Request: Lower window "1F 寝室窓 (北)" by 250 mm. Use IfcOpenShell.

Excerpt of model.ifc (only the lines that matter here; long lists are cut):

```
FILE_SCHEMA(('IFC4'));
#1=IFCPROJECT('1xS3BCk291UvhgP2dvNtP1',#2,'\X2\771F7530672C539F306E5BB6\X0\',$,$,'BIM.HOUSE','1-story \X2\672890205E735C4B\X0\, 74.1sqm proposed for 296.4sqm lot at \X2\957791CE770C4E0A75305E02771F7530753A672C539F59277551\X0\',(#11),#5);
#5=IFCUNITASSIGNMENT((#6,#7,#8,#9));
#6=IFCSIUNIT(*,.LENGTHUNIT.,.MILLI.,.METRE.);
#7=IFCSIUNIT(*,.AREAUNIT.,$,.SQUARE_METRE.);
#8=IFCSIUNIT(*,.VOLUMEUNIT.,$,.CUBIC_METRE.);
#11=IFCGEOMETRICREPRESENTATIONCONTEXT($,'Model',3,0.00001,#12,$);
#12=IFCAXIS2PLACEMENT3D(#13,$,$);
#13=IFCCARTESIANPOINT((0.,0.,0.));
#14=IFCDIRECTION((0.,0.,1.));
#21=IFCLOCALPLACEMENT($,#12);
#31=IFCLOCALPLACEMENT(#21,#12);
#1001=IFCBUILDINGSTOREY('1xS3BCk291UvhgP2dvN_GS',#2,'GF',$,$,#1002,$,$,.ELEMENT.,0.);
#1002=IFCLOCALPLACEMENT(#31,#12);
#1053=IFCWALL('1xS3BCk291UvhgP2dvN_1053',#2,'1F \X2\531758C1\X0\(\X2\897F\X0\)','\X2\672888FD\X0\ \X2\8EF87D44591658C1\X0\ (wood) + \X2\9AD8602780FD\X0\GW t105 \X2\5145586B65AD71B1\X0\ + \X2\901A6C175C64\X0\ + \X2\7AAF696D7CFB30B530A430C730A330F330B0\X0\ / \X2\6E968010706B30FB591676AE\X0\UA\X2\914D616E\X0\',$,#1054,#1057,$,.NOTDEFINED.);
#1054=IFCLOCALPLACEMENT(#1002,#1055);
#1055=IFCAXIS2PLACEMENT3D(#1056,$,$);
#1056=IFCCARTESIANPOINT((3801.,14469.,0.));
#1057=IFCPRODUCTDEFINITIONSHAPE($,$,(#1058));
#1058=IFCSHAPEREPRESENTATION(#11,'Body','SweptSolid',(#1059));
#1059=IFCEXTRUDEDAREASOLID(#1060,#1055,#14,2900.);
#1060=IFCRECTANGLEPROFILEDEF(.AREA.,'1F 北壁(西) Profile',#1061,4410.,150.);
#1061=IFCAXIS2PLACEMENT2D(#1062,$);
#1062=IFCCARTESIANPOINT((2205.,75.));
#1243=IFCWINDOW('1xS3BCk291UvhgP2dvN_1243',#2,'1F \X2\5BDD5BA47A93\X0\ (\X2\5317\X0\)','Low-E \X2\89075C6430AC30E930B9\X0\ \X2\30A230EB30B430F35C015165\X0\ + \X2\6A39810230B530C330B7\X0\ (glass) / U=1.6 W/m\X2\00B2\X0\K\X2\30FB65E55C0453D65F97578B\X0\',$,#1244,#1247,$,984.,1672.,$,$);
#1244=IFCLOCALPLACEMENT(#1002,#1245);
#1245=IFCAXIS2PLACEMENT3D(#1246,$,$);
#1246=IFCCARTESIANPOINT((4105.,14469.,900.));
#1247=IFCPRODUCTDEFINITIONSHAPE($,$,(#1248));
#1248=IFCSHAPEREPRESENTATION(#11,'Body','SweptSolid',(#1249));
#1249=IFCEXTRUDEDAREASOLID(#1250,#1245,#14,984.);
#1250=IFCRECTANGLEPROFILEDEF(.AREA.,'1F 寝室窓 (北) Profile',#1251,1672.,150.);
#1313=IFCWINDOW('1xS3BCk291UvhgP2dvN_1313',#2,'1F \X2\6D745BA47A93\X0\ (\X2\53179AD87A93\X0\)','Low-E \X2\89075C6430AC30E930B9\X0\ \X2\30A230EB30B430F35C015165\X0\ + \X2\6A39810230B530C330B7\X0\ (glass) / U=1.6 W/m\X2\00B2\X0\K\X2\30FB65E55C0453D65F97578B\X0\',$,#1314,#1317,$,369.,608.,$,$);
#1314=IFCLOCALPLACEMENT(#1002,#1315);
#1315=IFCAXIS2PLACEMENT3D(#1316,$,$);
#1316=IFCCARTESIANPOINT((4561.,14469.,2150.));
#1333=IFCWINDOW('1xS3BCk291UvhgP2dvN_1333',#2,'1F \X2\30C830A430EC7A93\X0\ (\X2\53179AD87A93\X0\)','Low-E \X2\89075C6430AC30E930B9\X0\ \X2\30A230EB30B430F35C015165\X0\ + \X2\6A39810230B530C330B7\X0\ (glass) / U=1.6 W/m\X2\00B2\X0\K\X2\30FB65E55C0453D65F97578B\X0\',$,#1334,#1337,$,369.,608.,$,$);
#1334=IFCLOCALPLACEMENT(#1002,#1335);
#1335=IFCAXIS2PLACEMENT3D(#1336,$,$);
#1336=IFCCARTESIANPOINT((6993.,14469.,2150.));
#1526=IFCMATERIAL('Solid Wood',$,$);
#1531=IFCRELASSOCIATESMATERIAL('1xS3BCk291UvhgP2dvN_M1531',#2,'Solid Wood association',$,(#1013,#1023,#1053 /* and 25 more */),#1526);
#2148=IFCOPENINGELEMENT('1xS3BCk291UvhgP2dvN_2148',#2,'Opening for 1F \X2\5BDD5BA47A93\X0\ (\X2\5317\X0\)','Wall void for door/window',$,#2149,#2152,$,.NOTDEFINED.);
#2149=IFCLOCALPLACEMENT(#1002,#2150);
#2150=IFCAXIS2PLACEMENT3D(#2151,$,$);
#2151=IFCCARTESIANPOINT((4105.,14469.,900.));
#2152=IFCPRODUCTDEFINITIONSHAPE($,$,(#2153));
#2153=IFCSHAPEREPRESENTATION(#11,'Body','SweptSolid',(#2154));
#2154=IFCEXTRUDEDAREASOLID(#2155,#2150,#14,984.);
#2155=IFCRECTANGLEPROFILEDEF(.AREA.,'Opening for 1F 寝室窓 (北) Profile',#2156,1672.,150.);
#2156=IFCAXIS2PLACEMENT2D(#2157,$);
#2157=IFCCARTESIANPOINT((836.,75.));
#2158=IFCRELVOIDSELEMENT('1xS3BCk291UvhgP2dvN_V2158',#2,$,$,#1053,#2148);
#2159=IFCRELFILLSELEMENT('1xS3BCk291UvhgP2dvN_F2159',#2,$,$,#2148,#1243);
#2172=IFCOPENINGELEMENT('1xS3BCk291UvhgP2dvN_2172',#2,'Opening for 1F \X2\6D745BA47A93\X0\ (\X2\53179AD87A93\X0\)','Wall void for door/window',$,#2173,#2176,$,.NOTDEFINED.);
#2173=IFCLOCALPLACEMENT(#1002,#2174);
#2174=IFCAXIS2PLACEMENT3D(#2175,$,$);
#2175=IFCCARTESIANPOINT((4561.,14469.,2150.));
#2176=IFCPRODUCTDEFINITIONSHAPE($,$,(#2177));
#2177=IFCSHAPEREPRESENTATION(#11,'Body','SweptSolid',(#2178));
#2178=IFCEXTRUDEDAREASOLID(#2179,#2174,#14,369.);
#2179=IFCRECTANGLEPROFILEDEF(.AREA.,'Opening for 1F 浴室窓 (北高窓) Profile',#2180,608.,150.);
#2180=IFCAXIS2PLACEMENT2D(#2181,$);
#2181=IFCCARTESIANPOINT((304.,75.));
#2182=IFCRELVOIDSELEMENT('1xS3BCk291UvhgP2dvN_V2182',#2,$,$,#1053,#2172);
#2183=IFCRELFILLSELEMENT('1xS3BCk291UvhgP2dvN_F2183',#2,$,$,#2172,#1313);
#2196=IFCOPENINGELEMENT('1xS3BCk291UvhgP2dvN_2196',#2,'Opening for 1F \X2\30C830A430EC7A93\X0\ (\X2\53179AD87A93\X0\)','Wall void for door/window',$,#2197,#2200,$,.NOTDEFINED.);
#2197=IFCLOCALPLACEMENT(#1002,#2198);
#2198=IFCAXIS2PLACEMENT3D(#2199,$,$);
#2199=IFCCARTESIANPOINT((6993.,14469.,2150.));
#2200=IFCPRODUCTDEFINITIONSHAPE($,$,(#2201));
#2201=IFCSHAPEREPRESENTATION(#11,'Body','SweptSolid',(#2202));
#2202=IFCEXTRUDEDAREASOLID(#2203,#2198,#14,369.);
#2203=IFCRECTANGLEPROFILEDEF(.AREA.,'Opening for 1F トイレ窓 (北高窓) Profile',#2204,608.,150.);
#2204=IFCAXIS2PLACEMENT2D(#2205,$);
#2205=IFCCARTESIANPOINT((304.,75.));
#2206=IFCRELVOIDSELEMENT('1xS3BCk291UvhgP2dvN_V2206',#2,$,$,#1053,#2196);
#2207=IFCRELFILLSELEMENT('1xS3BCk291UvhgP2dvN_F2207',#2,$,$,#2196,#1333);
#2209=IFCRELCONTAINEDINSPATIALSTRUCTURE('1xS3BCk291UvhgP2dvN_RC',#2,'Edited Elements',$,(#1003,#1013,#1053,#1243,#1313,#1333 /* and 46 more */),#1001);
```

```python
import numpy as np
import ifcopenshell
import ifcopenshell.api.geometry
import ifcopenshell.util.placement
import ifcopenshell.util.unit

model = ifcopenshell.open("model.ifc")
unit_scale = ifcopenshell.util.unit.calculate_unit_scale(model)

window = model.by_id(1243)
opening = window.FillsVoids[0].RelatingOpeningElement
dz = -250.0

shift = np.array([0.0, 0.0, dz])
# The window is not placed relative to its opening, so move both.
for product in (opening, window):
    matrix = ifcopenshell.util.placement.get_local_placement(product.ObjectPlacement)
    matrix[:3, 3] += shift
    ifcopenshell.api.geometry.edit_object_placement(model, product=product, matrix=matrix, is_si=False)

print(f"moved by {dz * unit_scale:+.3f} m")

model.write("model_updated.ifc")
```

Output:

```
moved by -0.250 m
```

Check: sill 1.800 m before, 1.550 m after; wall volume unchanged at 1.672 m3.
